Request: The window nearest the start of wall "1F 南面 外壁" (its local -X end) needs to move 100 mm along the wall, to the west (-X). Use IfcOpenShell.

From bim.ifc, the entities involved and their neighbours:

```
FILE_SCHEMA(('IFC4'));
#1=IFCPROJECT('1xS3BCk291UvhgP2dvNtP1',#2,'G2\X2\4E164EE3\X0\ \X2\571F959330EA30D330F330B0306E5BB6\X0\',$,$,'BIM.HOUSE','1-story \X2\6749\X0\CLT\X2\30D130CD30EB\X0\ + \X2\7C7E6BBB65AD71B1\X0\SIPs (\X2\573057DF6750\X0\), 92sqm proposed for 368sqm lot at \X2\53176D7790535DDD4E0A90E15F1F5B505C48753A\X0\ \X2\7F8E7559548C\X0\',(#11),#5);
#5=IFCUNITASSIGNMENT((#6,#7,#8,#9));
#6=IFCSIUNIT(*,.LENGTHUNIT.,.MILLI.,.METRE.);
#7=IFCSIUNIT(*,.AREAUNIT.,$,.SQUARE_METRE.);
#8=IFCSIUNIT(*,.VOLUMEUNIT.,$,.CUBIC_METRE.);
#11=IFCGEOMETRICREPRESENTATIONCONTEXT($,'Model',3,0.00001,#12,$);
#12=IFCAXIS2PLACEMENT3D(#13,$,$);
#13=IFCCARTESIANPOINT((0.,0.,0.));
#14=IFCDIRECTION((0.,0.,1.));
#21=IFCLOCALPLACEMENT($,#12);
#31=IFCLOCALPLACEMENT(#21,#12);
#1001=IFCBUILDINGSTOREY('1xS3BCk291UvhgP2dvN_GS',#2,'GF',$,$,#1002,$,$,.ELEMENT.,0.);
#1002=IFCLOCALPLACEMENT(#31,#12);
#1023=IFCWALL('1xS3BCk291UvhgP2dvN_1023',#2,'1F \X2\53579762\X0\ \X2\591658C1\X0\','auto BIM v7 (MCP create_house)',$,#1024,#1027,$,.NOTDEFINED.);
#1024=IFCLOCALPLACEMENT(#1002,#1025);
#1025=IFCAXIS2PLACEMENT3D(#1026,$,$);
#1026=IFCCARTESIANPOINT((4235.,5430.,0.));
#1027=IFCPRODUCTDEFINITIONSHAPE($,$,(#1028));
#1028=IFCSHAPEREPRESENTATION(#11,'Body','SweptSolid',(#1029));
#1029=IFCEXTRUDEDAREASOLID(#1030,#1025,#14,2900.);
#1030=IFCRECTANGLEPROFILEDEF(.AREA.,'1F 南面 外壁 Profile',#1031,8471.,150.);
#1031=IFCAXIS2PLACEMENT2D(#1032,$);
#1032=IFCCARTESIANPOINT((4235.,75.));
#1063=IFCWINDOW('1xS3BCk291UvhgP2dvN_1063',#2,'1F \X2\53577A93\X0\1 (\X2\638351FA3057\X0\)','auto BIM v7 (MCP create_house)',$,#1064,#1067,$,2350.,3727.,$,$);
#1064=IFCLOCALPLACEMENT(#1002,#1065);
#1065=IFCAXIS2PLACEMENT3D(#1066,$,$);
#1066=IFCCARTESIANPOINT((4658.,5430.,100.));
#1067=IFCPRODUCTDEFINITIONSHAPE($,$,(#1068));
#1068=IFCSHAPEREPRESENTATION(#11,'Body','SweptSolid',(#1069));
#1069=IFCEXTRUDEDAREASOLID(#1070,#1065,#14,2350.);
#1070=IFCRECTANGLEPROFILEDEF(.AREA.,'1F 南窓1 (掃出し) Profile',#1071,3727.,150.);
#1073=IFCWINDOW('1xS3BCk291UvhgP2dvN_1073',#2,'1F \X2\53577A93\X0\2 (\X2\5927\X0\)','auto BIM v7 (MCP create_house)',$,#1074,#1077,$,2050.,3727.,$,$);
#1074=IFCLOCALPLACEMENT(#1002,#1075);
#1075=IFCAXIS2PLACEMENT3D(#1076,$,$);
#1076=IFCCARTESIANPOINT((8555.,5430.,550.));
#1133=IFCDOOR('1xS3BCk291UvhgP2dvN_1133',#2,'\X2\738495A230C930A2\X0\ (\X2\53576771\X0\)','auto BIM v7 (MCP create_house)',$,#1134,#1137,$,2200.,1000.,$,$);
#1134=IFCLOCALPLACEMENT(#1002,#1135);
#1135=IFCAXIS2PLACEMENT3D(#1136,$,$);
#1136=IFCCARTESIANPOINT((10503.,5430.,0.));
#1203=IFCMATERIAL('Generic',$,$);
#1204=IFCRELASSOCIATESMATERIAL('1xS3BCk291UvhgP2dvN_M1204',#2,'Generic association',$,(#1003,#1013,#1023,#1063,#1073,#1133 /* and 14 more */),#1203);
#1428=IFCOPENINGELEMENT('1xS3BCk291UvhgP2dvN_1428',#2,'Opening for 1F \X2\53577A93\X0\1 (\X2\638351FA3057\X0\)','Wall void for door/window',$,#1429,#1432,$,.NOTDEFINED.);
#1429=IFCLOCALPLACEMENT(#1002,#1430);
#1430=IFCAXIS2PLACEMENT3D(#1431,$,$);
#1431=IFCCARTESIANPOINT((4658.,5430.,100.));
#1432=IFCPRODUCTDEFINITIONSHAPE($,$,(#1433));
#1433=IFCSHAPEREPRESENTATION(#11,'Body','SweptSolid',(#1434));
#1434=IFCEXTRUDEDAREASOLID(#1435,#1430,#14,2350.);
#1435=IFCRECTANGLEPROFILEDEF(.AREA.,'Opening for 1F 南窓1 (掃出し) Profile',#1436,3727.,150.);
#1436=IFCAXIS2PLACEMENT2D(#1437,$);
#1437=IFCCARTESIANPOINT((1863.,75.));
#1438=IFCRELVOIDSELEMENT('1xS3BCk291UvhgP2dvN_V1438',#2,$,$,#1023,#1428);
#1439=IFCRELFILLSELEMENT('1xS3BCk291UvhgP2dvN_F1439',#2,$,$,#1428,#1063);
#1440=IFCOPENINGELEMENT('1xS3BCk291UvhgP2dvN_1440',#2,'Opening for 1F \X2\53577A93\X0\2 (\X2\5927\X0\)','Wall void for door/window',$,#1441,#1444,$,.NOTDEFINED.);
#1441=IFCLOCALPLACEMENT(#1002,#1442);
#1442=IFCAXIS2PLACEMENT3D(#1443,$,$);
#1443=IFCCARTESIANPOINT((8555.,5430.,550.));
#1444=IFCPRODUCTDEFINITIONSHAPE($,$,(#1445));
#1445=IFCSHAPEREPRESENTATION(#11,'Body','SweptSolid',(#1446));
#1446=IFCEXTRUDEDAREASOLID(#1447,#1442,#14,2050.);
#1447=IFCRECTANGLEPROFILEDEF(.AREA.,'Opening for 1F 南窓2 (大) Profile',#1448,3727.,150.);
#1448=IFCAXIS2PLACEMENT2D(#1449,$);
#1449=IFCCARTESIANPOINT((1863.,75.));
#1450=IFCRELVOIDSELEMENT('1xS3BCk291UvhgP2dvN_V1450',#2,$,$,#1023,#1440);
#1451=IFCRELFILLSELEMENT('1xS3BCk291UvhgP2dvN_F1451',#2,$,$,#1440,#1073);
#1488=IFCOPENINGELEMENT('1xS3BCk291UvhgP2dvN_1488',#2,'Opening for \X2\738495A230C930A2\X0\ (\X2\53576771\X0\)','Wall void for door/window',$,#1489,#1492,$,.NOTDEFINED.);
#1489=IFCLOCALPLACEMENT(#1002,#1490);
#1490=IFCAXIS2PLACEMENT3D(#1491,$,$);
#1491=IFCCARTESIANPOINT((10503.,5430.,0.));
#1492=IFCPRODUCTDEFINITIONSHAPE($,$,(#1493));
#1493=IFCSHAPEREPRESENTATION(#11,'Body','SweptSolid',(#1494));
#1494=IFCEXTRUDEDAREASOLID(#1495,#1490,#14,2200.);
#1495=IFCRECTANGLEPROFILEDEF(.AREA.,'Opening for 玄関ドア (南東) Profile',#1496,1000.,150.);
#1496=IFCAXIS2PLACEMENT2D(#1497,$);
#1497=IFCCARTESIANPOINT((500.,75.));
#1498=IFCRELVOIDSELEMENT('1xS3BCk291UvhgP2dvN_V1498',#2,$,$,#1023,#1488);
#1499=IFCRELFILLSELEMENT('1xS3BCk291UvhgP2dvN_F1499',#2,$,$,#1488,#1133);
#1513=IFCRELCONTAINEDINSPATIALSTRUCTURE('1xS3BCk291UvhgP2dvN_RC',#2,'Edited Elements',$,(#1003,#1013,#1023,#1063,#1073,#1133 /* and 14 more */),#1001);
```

```python
import ifcopenshell
import ifcopenshell.api.geometry
import ifcopenshell.util.placement

model = ifcopenshell.open("bim.ifc")

window = model.by_guid("1xS3BCk291UvhgP2dvN_1063")
opening = window.FillsVoids[0].RelatingOpeningElement
wall = opening.VoidsElements[0].RelatingBuildingElement

wall_matrix = ifcopenshell.util.placement.get_local_placement(wall.ObjectPlacement)
shift = wall_matrix[:3, 0] * -100.0
before = ifcopenshell.util.placement.get_local_placement(window.ObjectPlacement)[:3, 3].copy()

# The window is not placed relative to its opening, so move both.
for product in (opening, window):
    matrix = ifcopenshell.util.placement.get_local_placement(product.ObjectPlacement)
    matrix[:3, 3] += shift
    ifcopenshell.api.geometry.edit_object_placement(model, product=product, matrix=matrix, is_si=False)

after = ifcopenshell.util.placement.get_local_placement(window.ObjectPlacement)[:3, 3]
print("window moved by", (after - before).round(3) + 0.0)

model.write("bim_updated.ifc")
```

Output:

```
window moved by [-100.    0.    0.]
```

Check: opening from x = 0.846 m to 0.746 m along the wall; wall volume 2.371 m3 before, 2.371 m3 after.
